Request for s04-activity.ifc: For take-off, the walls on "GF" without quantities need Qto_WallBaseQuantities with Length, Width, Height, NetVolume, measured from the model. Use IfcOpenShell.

First a look at what the model holds.

```python
import ifcopenshell
import ifcopenshell.util.element
import ifcopenshell.util.unit

model = ifcopenshell.open("s04-activity.ifc")
print(model.schema)
for unit_type in ("LENGTHUNIT", "AREAUNIT", "VOLUMEUNIT"):
    print(unit_type, ifcopenshell.util.unit.calculate_unit_scale(model, unit_type))
storey = next(s for s in model.by_type("IfcBuildingStorey") if s.Name == "GF")
walls = [e for e in ifcopenshell.util.element.get_decomposition(storey) if e.is_a("IfcWall")]
for e in sorted(walls, key=lambda e: e.id()):
    print(e.id(), e.is_a(), e.Name, list(ifcopenshell.util.element.get_psets(e, qtos_only=True)), sep=" | ")
```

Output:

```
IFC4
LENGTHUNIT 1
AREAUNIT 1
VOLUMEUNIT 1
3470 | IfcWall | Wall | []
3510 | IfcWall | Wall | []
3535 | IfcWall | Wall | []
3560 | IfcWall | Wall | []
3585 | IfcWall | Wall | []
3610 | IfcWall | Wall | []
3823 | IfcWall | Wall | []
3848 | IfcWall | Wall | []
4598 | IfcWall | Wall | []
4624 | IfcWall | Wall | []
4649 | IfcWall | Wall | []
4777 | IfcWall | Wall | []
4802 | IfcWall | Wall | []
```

```python
import ifcopenshell
import ifcopenshell.api.pset
import ifcopenshell.geom
import ifcopenshell.util.element
import ifcopenshell.util.shape
import ifcopenshell.util.unit

model = ifcopenshell.open("s04-activity.ifc")
unit_scale = ifcopenshell.util.unit.calculate_unit_scale(model)
volume_scale = ifcopenshell.util.unit.calculate_unit_scale(model, "VOLUMEUNIT")
settings = ifcopenshell.geom.settings()

storey = next(s for s in model.by_type("IfcBuildingStorey") if s.Name == "GF")
walls = [e for e in ifcopenshell.util.element.get_decomposition(storey) if e.is_a("IfcWall")]

for e in sorted(walls, key=lambda e: e.id()):
    if ifcopenshell.util.element.get_psets(e, qtos_only=True, should_inherit=False):
        continue
    # Geometry comes back in metres, in the element's own axes.
    shape = ifcopenshell.geom.create_shape(settings, e)
    values = {
        "Length": ifcopenshell.util.shape.get_x(shape.geometry) / unit_scale,
        "Width": ifcopenshell.util.shape.get_y(shape.geometry) / unit_scale,
        "Height": ifcopenshell.util.shape.get_z(shape.geometry) / unit_scale,
        "NetVolume": ifcopenshell.util.shape.get_volume(shape.geometry) / volume_scale,
    }
    qto = ifcopenshell.api.pset.add_qto(model, product=e, name="Qto_WallBaseQuantities")
    ifcopenshell.api.pset.edit_qto(model, qto=qto, properties=values)
    print(e.id(), {k: round(v, 3) for k, v in values.items()})

model.write("s04-activity_edited.ifc")
```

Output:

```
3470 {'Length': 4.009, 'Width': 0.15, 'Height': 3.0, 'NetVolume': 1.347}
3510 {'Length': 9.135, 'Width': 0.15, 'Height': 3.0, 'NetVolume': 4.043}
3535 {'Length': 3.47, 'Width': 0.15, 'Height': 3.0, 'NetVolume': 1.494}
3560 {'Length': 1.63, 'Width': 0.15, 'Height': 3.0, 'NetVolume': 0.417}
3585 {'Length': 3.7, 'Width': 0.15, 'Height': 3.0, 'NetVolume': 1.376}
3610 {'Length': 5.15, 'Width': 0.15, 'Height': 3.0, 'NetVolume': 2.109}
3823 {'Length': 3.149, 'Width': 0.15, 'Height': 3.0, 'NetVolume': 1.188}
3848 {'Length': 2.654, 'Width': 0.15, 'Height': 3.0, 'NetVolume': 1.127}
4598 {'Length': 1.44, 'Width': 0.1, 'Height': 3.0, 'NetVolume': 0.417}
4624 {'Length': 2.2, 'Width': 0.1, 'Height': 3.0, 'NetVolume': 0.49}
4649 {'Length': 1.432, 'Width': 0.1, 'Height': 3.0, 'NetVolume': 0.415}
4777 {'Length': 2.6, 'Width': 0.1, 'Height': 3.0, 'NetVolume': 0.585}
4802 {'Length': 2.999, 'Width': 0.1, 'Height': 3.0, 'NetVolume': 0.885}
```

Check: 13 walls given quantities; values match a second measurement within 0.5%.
